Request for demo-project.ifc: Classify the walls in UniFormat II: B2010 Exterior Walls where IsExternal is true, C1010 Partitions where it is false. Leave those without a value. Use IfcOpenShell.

First a look at what the model holds.

```python
import ifcopenshell
import ifcopenshell.util.element

model = ifcopenshell.open("demo-project.ifc")
print(model.schema)
print("classifications:", [c.Name for c in model.by_type("IfcClassification")])
values = [ifcopenshell.util.element.get_pset(e, "Pset_WallCommon", "IsExternal") for e in model.by_type("IfcWall")]
for value in (True, False, None):
    print("IsExternal", value, values.count(value))
```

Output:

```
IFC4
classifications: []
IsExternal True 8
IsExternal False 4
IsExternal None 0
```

```python
import ifcopenshell
import ifcopenshell.api.classification
import ifcopenshell.util.element

model = ifcopenshell.open("demo-project.ifc")

system = ifcopenshell.api.classification.add_classification(model, classification="UniFormat II")

walls = model.by_type("IfcWall")
external = {e: ifcopenshell.util.element.get_pset(e, "Pset_WallCommon", "IsExternal") for e in walls}
for flag, code, name in ((True, "B2010", "Exterior Walls"), (False, "C1010", "Partitions")):
    products = [e for e in walls if external[e] is flag]
    ifcopenshell.api.classification.add_reference(
        model, products=products, classification=system, identification=code, name=name
    )
    print(code, len(products))

model.write("demo-project_v2.ifc")
```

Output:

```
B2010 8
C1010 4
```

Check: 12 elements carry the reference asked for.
